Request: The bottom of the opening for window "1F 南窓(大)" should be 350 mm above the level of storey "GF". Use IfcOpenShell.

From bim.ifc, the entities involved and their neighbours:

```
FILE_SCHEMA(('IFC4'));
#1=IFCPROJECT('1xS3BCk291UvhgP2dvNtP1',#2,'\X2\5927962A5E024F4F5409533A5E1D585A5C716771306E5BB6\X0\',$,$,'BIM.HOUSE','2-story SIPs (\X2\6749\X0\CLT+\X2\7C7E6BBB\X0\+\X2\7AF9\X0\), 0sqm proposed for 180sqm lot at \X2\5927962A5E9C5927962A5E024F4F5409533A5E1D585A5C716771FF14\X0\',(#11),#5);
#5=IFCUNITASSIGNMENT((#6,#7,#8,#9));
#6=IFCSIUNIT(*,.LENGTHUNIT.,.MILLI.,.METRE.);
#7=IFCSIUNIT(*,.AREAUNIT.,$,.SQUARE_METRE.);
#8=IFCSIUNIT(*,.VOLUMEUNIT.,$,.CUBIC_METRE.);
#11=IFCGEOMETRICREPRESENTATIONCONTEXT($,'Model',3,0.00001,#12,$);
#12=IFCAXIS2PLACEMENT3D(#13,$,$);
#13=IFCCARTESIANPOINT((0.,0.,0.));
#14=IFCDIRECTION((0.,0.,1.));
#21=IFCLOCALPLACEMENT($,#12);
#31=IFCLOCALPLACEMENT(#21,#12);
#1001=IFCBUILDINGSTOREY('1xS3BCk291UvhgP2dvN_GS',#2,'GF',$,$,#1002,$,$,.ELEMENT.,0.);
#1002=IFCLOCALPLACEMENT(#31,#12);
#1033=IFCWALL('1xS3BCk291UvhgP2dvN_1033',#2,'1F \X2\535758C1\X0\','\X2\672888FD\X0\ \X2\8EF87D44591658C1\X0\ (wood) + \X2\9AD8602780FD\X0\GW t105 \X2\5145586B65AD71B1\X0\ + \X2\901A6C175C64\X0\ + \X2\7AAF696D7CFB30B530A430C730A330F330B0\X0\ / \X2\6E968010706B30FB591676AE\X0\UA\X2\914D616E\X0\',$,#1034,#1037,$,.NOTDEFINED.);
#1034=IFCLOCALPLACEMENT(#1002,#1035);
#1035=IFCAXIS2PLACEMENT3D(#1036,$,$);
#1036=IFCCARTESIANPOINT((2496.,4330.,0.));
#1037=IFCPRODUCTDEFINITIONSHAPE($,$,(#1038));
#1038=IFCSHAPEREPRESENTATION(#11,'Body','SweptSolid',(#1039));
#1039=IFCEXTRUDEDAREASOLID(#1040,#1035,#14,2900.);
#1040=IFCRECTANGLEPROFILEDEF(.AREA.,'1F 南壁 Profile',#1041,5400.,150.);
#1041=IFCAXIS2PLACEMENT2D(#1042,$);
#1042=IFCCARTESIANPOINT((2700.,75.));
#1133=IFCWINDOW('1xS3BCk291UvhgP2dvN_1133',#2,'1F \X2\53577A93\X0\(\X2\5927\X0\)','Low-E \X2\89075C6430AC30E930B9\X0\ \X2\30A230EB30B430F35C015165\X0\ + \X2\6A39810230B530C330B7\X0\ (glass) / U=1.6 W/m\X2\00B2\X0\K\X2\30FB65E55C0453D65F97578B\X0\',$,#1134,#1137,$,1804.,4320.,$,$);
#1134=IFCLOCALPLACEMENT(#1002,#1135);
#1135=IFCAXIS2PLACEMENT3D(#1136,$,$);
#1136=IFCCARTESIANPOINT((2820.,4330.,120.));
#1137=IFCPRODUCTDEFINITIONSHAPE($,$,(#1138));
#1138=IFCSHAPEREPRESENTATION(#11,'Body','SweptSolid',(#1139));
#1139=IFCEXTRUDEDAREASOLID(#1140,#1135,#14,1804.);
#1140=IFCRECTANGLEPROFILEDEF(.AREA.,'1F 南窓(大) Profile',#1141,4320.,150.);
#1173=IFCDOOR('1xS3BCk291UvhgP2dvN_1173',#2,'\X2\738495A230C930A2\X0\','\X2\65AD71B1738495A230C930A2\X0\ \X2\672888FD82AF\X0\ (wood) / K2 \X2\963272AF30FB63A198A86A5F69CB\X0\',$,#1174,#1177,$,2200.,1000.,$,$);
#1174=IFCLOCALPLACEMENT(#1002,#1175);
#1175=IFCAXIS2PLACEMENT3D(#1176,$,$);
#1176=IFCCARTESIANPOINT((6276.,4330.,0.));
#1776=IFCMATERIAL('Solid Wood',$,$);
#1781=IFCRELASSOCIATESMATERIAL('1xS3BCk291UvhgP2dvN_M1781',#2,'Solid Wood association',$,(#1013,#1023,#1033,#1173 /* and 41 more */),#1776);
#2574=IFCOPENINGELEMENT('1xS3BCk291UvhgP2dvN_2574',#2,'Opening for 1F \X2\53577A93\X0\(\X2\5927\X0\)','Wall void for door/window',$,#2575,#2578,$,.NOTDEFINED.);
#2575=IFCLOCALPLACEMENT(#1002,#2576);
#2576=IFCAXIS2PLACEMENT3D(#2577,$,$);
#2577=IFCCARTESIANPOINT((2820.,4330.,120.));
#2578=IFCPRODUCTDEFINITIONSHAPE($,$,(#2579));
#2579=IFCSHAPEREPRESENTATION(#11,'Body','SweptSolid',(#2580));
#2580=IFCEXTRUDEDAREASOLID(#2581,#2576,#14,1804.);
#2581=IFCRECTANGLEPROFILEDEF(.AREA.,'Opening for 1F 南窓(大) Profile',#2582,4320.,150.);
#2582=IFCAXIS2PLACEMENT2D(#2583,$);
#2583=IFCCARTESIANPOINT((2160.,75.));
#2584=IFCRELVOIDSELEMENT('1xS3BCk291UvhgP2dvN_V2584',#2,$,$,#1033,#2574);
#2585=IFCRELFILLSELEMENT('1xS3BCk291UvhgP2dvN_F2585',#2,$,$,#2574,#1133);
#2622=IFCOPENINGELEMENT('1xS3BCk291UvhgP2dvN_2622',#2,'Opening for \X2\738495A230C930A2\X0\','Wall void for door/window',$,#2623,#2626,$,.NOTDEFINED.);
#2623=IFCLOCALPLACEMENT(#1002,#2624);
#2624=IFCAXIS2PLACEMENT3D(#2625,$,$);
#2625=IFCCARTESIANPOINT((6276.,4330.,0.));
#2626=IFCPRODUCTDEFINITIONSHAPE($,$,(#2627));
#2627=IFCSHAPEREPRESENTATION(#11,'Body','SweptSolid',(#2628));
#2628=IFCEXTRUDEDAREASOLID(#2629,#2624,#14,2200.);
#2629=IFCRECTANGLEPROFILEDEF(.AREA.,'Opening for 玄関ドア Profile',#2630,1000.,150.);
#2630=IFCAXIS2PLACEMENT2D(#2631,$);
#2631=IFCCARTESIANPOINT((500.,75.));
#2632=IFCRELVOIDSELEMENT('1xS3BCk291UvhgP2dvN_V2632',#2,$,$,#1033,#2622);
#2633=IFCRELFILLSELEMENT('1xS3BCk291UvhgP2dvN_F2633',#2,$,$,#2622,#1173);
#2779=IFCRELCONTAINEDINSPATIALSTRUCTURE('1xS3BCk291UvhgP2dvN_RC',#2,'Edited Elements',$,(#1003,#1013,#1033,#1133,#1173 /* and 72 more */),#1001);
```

```python
import numpy as np
import ifcopenshell
import ifcopenshell.api.geometry
import ifcopenshell.geom
import ifcopenshell.util.element
import ifcopenshell.util.placement
import ifcopenshell.util.shape
import ifcopenshell.util.unit

model = ifcopenshell.open("bim.ifc")
unit_scale = ifcopenshell.util.unit.calculate_unit_scale(model)

window = model.by_id(1133)
opening = window.FillsVoids[0].RelatingOpeningElement
storey = ifcopenshell.util.element.get_container(window, ifc_class="IfcBuildingStorey")
level = ifcopenshell.util.placement.get_local_placement(storey.ObjectPlacement)[2, 3]

# The opening's origin need not be at the sill, so measure its lowest point.
shape = ifcopenshell.geom.create_shape(ifcopenshell.geom.settings(), opening)
bottom = ifcopenshell.util.shape.get_shape_bottom_elevation(shape, shape.geometry) / unit_scale
dz = level + 350.0 - bottom

shift = np.array([0.0, 0.0, dz])
# The window is not placed relative to its opening, so move both.
for product in (opening, window):
    matrix = ifcopenshell.util.placement.get_local_placement(product.ObjectPlacement)
    matrix[:3, 3] += shift
    ifcopenshell.api.geometry.edit_object_placement(model, product=product, matrix=matrix, is_si=False)

print(f"moved by {dz * unit_scale:+.3f} m")

model.write("bim_edited.ifc")
```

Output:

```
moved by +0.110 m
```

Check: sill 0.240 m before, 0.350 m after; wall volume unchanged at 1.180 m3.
